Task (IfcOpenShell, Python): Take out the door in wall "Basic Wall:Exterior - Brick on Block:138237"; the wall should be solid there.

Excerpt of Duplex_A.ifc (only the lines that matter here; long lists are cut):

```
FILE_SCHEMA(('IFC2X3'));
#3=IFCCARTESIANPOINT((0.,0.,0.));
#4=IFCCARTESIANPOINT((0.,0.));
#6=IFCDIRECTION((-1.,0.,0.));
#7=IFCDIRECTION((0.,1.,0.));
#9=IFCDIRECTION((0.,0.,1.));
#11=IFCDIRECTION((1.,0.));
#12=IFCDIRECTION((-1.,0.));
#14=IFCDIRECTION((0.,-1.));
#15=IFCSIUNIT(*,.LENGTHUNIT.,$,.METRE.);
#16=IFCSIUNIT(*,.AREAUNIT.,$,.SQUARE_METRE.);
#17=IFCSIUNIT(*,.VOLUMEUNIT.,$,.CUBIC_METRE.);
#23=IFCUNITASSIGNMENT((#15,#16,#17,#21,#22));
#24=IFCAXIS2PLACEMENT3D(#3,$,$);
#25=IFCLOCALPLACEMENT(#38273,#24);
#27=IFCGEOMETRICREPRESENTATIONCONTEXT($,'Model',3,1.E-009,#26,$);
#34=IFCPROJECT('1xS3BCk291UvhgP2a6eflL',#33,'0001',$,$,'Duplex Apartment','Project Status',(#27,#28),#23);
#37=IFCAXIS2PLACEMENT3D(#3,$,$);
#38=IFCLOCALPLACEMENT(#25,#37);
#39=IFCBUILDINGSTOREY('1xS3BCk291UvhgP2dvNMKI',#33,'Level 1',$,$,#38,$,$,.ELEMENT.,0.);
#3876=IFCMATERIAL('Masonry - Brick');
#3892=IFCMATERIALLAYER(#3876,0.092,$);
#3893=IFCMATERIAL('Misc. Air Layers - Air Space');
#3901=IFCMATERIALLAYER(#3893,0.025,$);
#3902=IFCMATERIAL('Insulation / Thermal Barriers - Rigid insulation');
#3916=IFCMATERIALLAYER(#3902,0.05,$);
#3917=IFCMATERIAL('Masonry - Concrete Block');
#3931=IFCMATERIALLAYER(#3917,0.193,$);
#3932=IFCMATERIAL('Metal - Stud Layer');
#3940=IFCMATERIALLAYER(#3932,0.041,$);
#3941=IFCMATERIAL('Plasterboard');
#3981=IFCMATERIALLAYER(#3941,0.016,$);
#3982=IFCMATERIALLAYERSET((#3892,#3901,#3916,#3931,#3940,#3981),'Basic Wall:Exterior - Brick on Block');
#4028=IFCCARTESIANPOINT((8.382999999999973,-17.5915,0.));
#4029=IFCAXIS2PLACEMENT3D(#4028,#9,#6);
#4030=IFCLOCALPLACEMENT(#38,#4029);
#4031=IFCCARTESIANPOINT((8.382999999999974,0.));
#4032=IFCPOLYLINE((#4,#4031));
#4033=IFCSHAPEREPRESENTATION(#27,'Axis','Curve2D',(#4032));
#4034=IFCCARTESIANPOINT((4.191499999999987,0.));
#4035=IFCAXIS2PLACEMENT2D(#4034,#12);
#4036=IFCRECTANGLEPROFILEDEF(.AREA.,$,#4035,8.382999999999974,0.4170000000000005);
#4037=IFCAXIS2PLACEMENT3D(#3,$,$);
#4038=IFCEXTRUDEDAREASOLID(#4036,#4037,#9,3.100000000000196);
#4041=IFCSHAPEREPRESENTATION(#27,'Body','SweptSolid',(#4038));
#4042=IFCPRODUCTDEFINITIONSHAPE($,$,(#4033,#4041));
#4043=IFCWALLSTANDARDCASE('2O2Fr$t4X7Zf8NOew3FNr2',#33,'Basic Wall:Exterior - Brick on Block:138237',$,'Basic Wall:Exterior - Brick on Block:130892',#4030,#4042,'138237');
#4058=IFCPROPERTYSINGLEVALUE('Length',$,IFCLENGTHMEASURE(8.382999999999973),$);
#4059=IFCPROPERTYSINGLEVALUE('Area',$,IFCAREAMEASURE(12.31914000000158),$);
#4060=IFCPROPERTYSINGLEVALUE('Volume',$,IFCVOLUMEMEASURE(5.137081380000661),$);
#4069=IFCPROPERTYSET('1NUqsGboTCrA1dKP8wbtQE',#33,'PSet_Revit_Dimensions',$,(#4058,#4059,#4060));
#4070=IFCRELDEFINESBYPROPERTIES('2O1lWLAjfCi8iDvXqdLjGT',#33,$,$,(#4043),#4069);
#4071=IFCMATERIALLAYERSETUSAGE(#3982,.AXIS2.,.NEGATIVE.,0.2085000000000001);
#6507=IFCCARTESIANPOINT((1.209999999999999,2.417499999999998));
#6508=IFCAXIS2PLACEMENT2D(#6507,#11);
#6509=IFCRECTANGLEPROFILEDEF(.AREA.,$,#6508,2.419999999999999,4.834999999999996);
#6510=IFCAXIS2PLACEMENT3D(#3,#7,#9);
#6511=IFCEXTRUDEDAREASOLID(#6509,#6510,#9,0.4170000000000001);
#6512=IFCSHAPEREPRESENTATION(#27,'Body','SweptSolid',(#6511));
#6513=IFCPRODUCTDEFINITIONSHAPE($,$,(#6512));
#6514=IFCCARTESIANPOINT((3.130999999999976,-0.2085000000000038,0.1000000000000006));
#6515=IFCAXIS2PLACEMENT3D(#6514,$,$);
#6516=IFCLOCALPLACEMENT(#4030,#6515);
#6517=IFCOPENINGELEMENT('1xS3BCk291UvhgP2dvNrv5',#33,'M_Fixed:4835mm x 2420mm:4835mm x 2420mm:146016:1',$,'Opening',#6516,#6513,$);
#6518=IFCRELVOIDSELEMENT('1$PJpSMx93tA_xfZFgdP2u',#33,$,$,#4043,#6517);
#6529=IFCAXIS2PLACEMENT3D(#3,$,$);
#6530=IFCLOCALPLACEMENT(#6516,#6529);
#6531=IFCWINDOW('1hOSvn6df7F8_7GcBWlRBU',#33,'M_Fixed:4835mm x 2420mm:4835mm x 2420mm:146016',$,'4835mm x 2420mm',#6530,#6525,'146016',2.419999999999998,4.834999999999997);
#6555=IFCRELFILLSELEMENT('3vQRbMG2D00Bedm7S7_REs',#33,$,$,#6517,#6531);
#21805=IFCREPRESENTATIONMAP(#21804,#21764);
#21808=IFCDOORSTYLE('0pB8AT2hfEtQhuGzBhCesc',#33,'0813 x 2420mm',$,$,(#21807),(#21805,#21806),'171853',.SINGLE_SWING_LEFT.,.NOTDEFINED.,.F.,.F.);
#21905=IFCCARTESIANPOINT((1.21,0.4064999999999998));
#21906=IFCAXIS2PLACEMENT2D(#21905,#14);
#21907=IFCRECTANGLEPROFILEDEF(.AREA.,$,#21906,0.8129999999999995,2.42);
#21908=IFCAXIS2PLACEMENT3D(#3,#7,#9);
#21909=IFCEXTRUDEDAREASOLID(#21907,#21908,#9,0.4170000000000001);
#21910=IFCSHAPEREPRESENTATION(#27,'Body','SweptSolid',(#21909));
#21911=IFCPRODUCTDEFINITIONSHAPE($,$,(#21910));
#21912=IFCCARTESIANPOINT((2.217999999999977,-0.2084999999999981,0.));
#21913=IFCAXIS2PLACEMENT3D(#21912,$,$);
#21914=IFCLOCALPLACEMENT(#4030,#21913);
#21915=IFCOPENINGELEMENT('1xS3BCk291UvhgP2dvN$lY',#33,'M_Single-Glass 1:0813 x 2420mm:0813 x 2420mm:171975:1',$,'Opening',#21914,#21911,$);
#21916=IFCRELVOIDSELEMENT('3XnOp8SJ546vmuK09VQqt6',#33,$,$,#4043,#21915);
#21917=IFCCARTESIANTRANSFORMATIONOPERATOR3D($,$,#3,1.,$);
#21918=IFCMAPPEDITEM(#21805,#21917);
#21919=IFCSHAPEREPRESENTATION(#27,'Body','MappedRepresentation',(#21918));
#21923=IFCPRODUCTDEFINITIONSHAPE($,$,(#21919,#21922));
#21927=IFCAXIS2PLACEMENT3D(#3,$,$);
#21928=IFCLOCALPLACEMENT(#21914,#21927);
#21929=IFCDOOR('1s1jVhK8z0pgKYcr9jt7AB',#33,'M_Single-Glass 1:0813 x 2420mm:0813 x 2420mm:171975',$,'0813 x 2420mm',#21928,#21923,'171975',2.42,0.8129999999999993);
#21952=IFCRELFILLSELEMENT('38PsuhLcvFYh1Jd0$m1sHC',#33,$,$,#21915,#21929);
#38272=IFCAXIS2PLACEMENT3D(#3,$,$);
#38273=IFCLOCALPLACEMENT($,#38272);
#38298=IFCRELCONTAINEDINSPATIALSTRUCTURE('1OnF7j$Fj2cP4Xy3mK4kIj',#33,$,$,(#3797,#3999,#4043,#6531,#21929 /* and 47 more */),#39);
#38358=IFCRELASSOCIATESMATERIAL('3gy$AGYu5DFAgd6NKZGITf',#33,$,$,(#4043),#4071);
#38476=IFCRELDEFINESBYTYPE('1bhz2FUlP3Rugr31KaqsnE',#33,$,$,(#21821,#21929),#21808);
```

```python
import ifcopenshell
import ifcopenshell.api.feature
import ifcopenshell.api.pset
import ifcopenshell.api.root
import ifcopenshell.geom
import ifcopenshell.util.element
import ifcopenshell.util.shape
import ifcopenshell.util.unit

model = ifcopenshell.open("Duplex_A.ifc")
area_scale = ifcopenshell.util.unit.calculate_unit_scale(model, "AREAUNIT")
volume_scale = ifcopenshell.util.unit.calculate_unit_scale(model, "VOLUMEUNIT")
settings = ifcopenshell.geom.settings()


def volume(element):
    """Net volume in cubic metres, openings subtracted."""
    shape = ifcopenshell.geom.create_shape(settings, element)
    return ifcopenshell.util.shape.get_volume(shape.geometry)


door = model.by_guid("1s1jVhK8z0pgKYcr9jt7AB")
opening = door.FillsVoids[0].RelatingOpeningElement
wall = opening.VoidsElements[0].RelatingBuildingElement
before = volume(wall)

ifcopenshell.api.root.remove_product(model, product=door)
ifcopenshell.api.feature.remove_feature(model, feature=opening)

after = volume(wall)
thickness = 0.417  # wall thickness in metres

# Update the wall's stored quantities.
pset = model.by_id(ifcopenshell.util.element.get_pset(wall, "PSet_Revit_Dimensions", should_inherit=False)["id"])
ifcopenshell.api.pset.edit_pset(model, pset=pset, properties={
    "Area": model.create_entity("IfcAreaMeasure", after / thickness / area_scale),
    "Volume": model.create_entity("IfcVolumeMeasure", after / volume_scale),
})

print(f"wall volume {before:.3f} -> {after:.3f} m3")

model.write("Duplex_A_rev.ifc")
```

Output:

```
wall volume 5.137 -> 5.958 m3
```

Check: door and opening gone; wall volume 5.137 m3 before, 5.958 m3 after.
